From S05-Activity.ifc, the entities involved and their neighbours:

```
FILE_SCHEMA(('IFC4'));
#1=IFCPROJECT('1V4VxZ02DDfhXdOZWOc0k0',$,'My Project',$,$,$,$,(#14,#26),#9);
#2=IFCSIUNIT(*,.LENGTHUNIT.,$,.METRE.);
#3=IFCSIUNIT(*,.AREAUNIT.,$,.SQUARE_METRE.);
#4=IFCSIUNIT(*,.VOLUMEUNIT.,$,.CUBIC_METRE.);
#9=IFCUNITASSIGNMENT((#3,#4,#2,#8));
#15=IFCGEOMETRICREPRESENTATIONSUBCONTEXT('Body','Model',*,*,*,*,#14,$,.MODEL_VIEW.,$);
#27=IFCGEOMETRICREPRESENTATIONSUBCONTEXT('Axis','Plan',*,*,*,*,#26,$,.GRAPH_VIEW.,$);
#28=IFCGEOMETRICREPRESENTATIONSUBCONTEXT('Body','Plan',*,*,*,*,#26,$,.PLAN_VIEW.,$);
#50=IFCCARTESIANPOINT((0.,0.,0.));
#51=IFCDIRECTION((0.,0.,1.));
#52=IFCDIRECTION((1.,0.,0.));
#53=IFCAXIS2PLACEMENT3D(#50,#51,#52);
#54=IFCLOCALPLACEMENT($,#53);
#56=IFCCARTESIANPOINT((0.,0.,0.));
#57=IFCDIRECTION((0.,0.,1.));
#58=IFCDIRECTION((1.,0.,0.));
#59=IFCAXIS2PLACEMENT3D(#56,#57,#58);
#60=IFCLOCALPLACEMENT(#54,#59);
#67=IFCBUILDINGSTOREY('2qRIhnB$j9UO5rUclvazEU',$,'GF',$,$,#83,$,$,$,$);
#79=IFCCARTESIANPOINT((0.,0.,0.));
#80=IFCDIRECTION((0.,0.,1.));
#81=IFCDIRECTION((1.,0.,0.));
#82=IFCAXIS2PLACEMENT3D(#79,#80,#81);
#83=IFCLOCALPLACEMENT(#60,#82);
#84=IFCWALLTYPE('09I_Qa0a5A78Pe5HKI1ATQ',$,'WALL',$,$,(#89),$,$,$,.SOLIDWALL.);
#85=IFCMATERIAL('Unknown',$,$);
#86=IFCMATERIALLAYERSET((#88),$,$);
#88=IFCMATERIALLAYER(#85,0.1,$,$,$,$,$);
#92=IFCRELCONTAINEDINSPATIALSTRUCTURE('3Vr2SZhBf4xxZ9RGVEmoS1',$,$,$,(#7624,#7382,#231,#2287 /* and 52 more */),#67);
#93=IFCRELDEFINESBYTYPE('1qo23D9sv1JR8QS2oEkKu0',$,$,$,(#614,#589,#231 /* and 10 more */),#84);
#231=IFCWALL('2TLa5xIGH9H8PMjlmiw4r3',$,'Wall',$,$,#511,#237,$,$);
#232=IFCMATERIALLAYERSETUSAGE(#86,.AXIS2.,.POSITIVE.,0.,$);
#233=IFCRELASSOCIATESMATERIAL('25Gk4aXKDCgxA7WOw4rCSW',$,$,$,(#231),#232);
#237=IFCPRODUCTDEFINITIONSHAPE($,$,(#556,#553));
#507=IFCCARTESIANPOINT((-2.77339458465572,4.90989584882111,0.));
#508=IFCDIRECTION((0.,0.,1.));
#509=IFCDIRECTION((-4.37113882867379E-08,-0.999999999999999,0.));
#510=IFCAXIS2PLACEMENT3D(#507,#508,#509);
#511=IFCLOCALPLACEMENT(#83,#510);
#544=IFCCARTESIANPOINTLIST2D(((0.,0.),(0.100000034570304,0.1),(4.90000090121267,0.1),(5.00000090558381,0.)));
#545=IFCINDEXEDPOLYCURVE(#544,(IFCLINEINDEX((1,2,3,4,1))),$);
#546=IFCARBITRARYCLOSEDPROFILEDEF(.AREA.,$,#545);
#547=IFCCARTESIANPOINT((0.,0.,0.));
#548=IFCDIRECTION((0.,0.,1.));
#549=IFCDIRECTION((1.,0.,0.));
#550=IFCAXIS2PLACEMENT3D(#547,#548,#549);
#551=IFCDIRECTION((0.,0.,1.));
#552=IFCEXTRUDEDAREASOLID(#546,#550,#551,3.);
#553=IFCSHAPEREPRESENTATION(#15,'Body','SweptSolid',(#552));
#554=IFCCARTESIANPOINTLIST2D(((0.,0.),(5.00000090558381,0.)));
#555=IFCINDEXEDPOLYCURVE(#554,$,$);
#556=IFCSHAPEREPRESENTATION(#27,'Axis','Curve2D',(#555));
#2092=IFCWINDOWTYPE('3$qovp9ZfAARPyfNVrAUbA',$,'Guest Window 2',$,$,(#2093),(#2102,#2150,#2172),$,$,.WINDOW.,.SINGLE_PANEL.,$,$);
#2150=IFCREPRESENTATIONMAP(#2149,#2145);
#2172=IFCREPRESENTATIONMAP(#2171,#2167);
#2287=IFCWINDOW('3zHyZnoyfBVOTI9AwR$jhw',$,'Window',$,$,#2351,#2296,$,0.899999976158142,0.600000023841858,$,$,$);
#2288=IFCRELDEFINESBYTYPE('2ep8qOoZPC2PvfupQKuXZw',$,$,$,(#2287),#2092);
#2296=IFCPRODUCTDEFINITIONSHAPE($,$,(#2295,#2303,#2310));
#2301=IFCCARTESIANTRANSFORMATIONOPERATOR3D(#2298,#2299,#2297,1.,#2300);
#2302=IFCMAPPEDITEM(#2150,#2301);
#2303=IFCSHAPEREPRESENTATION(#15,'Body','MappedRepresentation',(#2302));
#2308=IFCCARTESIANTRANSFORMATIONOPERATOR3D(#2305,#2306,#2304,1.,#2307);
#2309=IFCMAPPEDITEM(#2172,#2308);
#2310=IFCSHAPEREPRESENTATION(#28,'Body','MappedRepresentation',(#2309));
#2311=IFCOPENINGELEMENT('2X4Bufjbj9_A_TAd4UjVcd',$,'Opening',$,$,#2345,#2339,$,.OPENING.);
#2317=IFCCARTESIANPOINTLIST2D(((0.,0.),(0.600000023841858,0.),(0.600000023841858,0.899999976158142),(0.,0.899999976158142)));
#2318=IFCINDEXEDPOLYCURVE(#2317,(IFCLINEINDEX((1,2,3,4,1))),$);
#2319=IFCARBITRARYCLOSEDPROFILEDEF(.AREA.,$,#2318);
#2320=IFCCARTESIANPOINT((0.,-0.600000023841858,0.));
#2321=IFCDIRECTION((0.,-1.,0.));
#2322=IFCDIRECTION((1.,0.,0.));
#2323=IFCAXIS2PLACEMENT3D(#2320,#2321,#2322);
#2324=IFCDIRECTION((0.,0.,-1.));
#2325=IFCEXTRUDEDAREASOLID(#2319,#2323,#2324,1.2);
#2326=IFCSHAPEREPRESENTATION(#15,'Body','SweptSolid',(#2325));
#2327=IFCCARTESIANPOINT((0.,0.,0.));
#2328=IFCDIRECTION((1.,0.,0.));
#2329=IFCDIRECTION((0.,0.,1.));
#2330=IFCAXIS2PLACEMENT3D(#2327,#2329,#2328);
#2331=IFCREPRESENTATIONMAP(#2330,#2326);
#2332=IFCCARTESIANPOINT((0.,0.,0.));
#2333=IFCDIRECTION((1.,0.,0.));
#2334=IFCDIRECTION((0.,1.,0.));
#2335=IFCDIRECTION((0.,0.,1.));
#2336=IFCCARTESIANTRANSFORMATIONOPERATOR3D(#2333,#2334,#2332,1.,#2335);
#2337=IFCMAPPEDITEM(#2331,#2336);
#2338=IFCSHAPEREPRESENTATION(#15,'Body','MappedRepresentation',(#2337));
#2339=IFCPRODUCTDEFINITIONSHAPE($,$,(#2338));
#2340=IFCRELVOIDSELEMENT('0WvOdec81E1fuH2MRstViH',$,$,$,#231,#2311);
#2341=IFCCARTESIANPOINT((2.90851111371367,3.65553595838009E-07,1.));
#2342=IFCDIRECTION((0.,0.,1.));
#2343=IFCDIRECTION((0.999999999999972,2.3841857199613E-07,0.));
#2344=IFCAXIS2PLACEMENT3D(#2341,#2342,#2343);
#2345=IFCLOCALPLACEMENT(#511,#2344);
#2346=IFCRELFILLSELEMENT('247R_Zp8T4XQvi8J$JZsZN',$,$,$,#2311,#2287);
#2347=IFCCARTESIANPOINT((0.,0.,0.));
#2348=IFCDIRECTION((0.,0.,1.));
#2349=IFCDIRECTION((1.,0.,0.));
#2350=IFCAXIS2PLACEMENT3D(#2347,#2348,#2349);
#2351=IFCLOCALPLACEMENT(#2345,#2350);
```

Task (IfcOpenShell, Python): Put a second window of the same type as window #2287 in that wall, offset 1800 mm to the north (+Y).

```python
import ifcopenshell
import ifcopenshell.api.feature
import ifcopenshell.api.geometry
import ifcopenshell.api.root
import ifcopenshell.geom
import ifcopenshell.util.element
import ifcopenshell.util.placement
import ifcopenshell.util.shape
import ifcopenshell.util.unit

model = ifcopenshell.open("S05-Activity.ifc")
unit_scale = ifcopenshell.util.unit.calculate_unit_scale(model)
settings = ifcopenshell.geom.settings()


def volume(element):
    """Net volume in cubic metres, openings subtracted."""
    shape = ifcopenshell.geom.create_shape(settings, element)
    return ifcopenshell.util.shape.get_volume(shape.geometry)


window = model.by_id(2287)
opening = window.FillsVoids[0].RelatingOpeningElement
wall = opening.VoidsElements[0].RelatingBuildingElement
before = volume(wall)
shift = ifcopenshell.util.placement.get_local_placement(wall.ObjectPlacement)[:3, 0] * -1.8 / unit_scale

# copy_class copies the void relationship, type, container and properties, but no geometry.
new_opening = ifcopenshell.api.root.copy_class(model, product=opening)
new_opening.Representation = ifcopenshell.util.element.copy_deep(
    model, opening.Representation, exclude=["IfcGeometricRepresentationContext", "IfcRepresentationMap"]
)
new_window = ifcopenshell.api.root.copy_class(model, product=window)
new_window.Representation = ifcopenshell.util.element.copy_deep(
    model, window.Representation, exclude=["IfcGeometricRepresentationContext", "IfcRepresentationMap"]
)
ifcopenshell.api.feature.add_filling(model, opening=new_opening, element=new_window)

for old, new in ((opening, new_opening), (window, new_window)):
    matrix = ifcopenshell.util.placement.get_local_placement(old.ObjectPlacement)
    matrix[:3, 3] += shift
    ifcopenshell.api.geometry.edit_object_placement(model, product=new, matrix=matrix, is_si=False)

after = volume(wall)

print(f"wall volume {before:.3f} -> {after:.3f} m3")

model.write("S05-Activity_rev.ifc")
```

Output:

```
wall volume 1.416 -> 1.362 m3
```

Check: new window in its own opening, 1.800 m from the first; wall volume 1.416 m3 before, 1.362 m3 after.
